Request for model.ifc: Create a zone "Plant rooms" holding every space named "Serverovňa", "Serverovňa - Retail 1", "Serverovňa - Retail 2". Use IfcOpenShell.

First a look at what the model holds.

```python
import ifcopenshell

model = ifcopenshell.open("model.ifc")
print(model.schema)
seen = {}
for space in model.by_type("IfcSpace"):
    seen[space.LongName] = seen.get(space.LongName, 0) + 1
for name, count in sorted(seen.items(), key=str):
    print(count, "x", name)
print("zones:", [z.Name for z in model.by_type("IfcZone")][:20])
```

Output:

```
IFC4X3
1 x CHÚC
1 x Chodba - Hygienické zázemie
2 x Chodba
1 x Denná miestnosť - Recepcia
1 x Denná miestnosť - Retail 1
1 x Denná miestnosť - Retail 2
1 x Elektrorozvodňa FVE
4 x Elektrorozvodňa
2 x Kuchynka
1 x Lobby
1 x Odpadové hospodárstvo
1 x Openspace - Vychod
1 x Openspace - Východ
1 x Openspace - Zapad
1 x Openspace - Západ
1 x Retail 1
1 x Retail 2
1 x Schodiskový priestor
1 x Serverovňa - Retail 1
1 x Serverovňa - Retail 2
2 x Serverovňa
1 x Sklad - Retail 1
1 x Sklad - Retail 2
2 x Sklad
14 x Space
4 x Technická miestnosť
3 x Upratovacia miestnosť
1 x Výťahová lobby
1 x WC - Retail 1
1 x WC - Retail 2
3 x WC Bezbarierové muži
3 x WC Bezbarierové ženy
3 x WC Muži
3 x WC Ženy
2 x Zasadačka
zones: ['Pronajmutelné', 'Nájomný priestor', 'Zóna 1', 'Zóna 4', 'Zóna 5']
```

```python
import ifcopenshell
import ifcopenshell.api.group
import ifcopenshell.api.root

model = ifcopenshell.open("model.ifc")

names = {"Serverovňa", "Serverovňa - Retail 1", "Serverovňa - Retail 2"}
spaces = [s for s in model.by_type("IfcSpace") if s.LongName in names]

zone = ifcopenshell.api.root.create_entity(model, ifc_class="IfcZone", name="Plant rooms")
ifcopenshell.api.group.assign_group(model, products=spaces, group=zone)
print(len(spaces), "spaces in", zone.Name)

model.write("model-out.ifc")
```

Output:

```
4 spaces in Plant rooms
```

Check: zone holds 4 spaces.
